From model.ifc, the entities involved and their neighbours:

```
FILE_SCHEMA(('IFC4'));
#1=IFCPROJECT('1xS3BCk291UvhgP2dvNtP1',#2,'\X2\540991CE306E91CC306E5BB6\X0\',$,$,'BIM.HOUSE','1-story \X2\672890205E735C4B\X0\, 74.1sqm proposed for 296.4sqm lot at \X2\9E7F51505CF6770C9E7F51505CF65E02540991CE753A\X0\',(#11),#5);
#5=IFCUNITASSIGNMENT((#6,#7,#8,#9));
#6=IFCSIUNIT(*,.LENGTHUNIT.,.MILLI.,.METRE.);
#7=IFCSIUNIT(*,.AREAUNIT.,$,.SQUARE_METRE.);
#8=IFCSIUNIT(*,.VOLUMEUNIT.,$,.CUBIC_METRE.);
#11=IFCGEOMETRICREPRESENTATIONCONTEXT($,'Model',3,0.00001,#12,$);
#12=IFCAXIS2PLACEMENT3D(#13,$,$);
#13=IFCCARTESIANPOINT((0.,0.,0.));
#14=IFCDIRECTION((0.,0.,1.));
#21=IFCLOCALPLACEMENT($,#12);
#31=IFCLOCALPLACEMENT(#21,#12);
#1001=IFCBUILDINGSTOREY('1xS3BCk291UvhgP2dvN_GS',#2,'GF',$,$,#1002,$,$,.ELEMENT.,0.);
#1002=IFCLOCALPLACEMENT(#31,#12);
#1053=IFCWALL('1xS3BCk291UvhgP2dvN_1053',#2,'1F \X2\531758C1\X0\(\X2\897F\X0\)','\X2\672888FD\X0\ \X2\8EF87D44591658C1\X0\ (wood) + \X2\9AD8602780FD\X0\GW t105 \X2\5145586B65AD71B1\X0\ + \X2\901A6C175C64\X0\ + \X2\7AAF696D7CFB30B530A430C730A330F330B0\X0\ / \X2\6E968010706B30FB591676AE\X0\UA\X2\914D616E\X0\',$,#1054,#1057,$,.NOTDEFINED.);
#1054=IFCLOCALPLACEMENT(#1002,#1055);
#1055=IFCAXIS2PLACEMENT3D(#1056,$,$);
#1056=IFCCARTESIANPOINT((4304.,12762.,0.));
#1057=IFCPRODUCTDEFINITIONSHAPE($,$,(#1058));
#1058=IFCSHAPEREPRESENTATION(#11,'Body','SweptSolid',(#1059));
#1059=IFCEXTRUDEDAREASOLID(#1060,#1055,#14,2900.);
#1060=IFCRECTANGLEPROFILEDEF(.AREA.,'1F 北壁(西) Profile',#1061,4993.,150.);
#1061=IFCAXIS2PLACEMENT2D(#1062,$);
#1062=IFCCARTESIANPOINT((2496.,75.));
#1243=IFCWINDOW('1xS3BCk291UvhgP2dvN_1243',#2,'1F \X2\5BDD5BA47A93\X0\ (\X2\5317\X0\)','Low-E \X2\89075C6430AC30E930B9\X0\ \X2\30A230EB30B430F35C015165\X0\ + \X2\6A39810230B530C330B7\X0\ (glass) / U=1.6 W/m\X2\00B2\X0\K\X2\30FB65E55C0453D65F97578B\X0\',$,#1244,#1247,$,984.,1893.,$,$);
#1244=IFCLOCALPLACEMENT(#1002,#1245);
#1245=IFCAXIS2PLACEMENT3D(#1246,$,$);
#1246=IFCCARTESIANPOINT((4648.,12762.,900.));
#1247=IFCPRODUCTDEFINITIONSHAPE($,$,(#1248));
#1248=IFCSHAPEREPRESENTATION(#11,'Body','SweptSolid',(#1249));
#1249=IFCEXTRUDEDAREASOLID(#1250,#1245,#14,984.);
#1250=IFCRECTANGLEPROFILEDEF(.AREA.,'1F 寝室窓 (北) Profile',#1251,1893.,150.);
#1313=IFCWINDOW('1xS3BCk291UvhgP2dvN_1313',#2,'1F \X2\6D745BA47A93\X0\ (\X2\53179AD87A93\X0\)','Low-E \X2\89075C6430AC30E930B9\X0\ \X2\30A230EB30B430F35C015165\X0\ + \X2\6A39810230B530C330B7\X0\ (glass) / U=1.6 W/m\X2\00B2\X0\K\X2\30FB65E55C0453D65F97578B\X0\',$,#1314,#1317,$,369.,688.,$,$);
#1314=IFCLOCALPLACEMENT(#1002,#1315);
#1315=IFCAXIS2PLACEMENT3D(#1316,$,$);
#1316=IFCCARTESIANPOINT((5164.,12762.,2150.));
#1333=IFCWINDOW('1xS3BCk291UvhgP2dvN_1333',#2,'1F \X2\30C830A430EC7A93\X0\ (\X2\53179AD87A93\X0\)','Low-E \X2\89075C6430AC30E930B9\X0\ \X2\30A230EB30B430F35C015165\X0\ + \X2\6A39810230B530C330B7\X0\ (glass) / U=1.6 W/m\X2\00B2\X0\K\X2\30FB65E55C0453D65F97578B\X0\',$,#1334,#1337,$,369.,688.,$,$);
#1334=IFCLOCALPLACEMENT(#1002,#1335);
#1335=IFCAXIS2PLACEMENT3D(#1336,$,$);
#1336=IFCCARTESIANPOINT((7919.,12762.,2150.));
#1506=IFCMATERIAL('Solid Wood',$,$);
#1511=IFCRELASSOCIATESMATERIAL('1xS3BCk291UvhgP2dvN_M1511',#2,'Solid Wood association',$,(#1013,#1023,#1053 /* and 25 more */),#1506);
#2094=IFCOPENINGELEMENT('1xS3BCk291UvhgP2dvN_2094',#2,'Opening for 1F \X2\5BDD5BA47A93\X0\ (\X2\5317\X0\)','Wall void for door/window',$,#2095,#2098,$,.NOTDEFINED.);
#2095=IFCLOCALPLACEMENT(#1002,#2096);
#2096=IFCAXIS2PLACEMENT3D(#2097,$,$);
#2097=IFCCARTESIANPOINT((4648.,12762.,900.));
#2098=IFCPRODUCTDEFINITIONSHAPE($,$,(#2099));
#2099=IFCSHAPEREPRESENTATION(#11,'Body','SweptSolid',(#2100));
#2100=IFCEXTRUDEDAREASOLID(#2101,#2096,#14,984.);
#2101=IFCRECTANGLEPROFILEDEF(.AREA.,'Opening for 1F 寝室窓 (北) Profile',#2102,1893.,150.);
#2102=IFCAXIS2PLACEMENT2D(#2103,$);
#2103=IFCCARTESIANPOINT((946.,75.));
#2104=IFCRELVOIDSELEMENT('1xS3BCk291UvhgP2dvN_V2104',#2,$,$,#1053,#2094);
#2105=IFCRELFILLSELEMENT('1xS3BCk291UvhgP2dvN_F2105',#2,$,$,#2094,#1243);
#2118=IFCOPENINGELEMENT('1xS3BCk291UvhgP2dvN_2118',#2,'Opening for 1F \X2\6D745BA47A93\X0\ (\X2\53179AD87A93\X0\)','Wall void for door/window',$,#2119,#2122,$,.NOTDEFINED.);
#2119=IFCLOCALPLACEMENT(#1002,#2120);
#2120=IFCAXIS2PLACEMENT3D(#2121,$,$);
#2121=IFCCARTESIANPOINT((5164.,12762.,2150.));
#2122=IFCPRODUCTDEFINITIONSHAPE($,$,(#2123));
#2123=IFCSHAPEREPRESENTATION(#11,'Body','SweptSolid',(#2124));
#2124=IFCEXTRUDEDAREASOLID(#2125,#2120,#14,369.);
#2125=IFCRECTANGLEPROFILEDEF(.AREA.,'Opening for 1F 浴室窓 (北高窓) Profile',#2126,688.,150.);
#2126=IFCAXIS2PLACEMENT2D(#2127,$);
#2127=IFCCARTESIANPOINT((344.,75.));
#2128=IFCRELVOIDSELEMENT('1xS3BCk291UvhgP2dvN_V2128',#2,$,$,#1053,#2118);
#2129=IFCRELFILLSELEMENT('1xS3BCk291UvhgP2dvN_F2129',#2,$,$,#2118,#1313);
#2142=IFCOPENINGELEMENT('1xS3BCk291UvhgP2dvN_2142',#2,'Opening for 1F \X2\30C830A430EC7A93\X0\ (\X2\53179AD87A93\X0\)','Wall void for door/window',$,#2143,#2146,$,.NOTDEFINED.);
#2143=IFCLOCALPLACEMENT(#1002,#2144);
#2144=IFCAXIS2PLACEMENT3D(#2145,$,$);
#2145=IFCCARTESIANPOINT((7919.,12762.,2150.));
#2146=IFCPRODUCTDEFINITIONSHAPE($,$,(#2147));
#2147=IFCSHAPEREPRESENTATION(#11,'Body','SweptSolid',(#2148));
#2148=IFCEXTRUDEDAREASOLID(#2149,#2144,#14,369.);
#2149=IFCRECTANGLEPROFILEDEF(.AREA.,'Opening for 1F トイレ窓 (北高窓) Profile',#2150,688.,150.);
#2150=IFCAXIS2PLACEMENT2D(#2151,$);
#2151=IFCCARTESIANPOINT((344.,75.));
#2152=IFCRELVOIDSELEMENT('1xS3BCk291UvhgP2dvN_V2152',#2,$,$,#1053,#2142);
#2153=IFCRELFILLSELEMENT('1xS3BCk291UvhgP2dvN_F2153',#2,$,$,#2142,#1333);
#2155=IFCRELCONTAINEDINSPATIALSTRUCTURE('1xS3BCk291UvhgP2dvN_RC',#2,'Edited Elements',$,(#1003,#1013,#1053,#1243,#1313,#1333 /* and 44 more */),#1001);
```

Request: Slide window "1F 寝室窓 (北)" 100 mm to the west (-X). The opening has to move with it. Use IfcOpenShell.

```python
import ifcopenshell
import ifcopenshell.api.geometry
import ifcopenshell.util.placement

model = ifcopenshell.open("model.ifc")

window = model.by_guid("1xS3BCk291UvhgP2dvN_1243")
opening = window.FillsVoids[0].RelatingOpeningElement
wall = opening.VoidsElements[0].RelatingBuildingElement

wall_matrix = ifcopenshell.util.placement.get_local_placement(wall.ObjectPlacement)
shift = wall_matrix[:3, 0] * -100.0
before = ifcopenshell.util.placement.get_local_placement(window.ObjectPlacement)[:3, 3].copy()

# The window is not placed relative to its opening, so move both.
for product in (opening, window):
    matrix = ifcopenshell.util.placement.get_local_placement(product.ObjectPlacement)
    matrix[:3, 3] += shift
    ifcopenshell.api.geometry.edit_object_placement(model, product=product, matrix=matrix, is_si=False)

after = ifcopenshell.util.placement.get_local_placement(window.ObjectPlacement)[:3, 3]
print("window moved by", (after - before).round(3) + 0.0)

model.write("model-out.ifc")
```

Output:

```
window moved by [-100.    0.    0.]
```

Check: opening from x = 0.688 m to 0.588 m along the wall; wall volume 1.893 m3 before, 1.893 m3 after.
